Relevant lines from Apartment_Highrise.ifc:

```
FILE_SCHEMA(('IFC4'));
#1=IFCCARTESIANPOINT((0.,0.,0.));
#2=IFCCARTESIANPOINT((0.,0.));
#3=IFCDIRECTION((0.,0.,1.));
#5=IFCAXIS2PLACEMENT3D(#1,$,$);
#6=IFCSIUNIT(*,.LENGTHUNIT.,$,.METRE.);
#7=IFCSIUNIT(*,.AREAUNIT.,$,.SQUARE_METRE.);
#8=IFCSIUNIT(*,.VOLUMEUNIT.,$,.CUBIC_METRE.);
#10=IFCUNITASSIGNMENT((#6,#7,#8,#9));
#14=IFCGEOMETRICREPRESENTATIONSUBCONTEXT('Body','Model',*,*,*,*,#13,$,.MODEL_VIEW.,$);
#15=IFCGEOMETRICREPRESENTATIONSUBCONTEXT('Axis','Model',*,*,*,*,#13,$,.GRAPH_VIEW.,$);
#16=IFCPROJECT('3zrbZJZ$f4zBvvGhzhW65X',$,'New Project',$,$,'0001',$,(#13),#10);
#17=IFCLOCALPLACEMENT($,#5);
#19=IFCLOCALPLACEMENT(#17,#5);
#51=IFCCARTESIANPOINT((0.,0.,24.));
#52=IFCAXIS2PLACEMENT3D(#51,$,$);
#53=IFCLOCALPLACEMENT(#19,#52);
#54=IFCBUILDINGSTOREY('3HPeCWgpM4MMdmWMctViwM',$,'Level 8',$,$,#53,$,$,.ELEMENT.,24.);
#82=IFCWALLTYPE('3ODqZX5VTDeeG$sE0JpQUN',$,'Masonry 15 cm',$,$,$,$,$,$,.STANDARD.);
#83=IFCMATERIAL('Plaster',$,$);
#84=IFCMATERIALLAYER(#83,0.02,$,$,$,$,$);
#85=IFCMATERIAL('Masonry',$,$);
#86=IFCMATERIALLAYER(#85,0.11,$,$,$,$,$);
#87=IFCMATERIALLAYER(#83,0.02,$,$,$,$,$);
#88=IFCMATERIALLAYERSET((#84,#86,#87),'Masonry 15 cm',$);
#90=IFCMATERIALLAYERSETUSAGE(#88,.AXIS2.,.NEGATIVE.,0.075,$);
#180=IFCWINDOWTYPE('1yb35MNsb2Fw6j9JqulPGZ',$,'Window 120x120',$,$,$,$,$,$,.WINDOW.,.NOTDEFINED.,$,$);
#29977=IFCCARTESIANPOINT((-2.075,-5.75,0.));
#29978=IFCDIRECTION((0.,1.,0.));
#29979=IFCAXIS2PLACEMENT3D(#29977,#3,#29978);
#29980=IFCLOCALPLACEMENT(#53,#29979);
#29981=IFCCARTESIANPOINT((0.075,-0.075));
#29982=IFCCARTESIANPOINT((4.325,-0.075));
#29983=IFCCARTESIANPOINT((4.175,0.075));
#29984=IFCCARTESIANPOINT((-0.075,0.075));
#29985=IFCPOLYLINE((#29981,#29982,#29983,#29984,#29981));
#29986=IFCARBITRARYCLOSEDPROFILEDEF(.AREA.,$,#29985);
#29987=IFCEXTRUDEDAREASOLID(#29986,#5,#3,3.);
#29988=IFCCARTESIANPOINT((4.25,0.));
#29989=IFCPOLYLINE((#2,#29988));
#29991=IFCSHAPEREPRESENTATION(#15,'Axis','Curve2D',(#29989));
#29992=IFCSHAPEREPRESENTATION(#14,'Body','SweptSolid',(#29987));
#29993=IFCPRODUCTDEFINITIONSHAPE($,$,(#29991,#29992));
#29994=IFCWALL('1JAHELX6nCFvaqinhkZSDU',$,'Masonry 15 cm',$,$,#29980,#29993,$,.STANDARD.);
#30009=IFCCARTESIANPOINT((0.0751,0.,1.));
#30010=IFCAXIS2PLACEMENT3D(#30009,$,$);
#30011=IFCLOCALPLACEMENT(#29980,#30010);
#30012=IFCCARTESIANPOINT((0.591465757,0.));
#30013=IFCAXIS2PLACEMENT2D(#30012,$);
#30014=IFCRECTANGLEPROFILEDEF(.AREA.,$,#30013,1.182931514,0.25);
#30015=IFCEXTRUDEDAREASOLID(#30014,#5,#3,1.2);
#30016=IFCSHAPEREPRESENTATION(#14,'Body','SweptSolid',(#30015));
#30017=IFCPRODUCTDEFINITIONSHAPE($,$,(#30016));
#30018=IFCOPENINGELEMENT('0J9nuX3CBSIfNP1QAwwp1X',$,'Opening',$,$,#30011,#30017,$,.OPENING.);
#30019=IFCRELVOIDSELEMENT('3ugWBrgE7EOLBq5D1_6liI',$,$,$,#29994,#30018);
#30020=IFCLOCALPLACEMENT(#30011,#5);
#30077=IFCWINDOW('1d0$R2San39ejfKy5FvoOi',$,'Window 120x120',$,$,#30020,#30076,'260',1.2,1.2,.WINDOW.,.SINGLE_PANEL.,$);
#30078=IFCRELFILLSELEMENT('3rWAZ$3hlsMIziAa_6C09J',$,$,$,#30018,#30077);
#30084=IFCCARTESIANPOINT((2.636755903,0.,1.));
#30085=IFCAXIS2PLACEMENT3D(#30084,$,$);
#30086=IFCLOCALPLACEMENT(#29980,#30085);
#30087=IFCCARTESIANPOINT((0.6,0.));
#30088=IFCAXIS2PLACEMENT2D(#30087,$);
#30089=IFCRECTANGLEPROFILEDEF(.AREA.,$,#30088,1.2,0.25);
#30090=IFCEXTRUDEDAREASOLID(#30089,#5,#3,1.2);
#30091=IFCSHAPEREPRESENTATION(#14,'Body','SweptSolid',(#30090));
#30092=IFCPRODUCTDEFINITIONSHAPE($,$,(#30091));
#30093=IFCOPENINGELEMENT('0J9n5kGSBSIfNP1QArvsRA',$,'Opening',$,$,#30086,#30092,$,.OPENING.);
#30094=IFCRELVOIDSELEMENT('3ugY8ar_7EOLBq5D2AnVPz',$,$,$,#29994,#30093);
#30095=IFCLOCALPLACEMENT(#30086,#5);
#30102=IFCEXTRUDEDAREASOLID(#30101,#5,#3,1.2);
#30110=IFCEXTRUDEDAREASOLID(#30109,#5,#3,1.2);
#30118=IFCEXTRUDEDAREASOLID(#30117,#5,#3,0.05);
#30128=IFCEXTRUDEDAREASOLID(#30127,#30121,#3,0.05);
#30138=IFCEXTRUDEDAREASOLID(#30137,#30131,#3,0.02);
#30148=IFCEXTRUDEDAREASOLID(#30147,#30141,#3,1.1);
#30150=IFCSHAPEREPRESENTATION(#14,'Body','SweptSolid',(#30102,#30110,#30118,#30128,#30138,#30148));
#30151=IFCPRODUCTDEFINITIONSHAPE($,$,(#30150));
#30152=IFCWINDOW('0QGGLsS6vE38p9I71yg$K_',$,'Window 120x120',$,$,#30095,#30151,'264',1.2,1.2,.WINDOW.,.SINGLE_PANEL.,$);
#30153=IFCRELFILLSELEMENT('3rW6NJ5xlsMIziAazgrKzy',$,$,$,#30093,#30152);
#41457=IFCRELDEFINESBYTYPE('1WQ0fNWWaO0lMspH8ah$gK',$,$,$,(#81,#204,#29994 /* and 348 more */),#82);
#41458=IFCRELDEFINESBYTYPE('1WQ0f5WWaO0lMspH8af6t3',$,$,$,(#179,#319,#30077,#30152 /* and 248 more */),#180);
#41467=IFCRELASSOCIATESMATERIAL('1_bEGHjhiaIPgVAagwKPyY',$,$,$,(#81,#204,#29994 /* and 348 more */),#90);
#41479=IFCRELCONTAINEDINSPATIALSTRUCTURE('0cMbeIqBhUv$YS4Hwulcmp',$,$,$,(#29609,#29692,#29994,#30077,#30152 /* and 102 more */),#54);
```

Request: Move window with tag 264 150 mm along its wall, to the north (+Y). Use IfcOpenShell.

```python
import ifcopenshell
import ifcopenshell.api.geometry
import ifcopenshell.util.placement
import ifcopenshell.util.unit

model = ifcopenshell.open("Apartment_Highrise.ifc")
unit_scale = ifcopenshell.util.unit.calculate_unit_scale(model)

window = model.by_guid("0QGGLsS6vE38p9I71yg$K_")
opening = window.FillsVoids[0].RelatingOpeningElement
wall = opening.VoidsElements[0].RelatingBuildingElement

wall_matrix = ifcopenshell.util.placement.get_local_placement(wall.ObjectPlacement)
shift = wall_matrix[:3, 0] * 0.15 / unit_scale
before = ifcopenshell.util.placement.get_local_placement(window.ObjectPlacement)[:3, 3].copy()

# The window is placed relative to its opening, so it follows when the opening moves.
matrix = ifcopenshell.util.placement.get_local_placement(opening.ObjectPlacement)
matrix[:3, 3] += shift
ifcopenshell.api.geometry.edit_object_placement(
    model, product=opening, matrix=matrix, is_si=False, should_transform_children=True
)

after = ifcopenshell.util.placement.get_local_placement(window.ObjectPlacement)[:3, 3]
print("window moved by", (after - before).round(3) + 0.0)

model.write("Apartment_Highrise_rev.ifc")
```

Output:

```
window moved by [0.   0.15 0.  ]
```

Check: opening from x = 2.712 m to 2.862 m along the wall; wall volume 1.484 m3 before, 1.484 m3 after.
